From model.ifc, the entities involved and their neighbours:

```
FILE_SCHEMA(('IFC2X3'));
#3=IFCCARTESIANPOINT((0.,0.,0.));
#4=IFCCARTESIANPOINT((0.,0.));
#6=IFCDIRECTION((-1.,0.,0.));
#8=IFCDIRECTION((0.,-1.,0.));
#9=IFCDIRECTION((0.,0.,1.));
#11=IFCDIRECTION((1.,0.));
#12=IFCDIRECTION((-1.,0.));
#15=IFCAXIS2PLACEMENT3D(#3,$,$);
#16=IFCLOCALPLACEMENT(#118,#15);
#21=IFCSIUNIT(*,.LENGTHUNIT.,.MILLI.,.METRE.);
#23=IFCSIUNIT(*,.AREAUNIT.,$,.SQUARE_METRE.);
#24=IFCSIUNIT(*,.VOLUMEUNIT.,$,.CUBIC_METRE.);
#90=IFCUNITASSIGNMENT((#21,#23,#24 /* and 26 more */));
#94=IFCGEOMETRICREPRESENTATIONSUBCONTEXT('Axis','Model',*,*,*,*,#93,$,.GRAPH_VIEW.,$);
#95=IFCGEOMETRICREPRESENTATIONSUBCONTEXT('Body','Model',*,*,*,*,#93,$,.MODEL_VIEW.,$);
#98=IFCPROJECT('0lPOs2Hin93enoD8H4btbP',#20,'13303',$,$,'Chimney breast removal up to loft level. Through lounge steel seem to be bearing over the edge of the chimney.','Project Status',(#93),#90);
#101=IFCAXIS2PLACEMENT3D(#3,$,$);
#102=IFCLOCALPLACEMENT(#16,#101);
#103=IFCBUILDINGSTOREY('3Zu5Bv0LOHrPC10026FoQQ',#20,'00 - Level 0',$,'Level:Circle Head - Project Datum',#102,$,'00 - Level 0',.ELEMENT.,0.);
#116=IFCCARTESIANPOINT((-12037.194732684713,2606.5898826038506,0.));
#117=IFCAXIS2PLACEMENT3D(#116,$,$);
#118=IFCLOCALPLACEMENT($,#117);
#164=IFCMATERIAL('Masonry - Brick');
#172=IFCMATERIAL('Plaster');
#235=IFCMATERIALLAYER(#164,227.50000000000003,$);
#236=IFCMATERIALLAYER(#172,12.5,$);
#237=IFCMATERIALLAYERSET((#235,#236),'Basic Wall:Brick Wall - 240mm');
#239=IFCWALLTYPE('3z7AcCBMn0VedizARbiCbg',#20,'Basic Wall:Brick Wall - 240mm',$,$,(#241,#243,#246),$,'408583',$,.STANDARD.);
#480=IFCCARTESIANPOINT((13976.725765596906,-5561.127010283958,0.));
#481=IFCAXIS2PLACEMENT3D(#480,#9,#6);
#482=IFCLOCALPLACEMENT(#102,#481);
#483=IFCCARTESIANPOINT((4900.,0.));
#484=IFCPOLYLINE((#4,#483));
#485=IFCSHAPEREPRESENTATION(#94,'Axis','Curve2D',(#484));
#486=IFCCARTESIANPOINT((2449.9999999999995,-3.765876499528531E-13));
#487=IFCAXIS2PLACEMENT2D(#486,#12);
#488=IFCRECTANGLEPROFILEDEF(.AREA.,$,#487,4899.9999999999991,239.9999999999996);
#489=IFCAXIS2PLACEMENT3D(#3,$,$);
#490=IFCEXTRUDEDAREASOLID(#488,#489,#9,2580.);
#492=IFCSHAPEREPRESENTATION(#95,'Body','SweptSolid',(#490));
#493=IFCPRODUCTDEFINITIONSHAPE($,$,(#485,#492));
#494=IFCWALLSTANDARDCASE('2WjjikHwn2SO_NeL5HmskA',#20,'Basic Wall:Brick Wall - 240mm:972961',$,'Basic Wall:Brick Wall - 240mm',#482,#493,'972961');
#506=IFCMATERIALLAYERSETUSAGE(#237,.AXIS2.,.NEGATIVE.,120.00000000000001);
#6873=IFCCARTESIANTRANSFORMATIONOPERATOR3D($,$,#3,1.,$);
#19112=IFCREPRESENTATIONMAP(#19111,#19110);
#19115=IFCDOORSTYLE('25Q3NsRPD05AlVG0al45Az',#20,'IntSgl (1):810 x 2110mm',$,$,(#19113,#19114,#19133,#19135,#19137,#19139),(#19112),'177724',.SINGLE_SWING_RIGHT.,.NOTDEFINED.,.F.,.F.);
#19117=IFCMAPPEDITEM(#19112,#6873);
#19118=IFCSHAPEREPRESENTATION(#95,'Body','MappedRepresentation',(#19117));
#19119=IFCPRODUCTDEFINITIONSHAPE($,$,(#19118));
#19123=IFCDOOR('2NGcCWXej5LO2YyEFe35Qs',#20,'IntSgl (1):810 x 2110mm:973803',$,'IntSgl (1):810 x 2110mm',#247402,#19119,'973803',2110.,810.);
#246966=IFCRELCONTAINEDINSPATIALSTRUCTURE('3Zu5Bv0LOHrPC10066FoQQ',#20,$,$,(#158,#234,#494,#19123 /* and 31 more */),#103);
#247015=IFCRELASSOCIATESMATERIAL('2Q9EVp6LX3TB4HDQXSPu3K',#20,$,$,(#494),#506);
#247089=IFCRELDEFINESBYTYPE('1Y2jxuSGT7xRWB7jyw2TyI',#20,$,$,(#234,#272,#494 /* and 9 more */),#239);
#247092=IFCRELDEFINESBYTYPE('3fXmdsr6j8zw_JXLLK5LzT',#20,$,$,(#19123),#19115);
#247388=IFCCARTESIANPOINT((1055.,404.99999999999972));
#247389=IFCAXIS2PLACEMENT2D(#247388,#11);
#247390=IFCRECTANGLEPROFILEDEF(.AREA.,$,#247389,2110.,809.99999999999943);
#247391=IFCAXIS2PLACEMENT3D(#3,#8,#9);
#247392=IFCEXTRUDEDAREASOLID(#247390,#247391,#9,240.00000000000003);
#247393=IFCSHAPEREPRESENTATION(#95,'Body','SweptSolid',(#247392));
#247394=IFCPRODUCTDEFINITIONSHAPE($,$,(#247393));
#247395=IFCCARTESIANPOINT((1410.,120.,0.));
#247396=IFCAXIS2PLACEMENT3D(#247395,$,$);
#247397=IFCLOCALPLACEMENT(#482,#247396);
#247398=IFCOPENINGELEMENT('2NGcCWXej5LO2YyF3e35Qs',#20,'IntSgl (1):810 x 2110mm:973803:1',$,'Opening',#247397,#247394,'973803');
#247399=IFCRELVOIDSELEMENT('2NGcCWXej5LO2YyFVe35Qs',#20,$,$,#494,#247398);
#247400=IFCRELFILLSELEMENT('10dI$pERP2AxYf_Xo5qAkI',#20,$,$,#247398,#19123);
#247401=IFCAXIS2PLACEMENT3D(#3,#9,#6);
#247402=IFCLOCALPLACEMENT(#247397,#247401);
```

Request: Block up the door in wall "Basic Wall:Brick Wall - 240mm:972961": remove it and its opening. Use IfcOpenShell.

```python
import ifcopenshell
import ifcopenshell.api.feature
import ifcopenshell.api.root
import ifcopenshell.geom
import ifcopenshell.util.shape

model = ifcopenshell.open("model.ifc")
settings = ifcopenshell.geom.settings()


def volume(element):
    """Net volume in cubic metres, openings subtracted."""
    shape = ifcopenshell.geom.create_shape(settings, element)
    return ifcopenshell.util.shape.get_volume(shape.geometry)


door = model.by_guid("2NGcCWXej5LO2YyEFe35Qs")
opening = door.FillsVoids[0].RelatingOpeningElement
wall = opening.VoidsElements[0].RelatingBuildingElement
before = volume(wall)

ifcopenshell.api.root.remove_product(model, product=door)
ifcopenshell.api.feature.remove_feature(model, feature=opening)

after = volume(wall)

print(f"wall volume {before:.3f} -> {after:.3f} m3")

model.write("model-out.ifc")
```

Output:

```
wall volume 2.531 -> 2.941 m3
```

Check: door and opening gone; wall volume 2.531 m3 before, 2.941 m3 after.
